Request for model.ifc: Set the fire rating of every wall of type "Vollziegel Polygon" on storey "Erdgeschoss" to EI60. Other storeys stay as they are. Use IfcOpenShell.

First a look at what the model holds.

```python
import ifcopenshell
import ifcopenshell.util.element

model = ifcopenshell.open("model.ifc")
print(model.schema)
storey = next(s for s in model.by_type("IfcBuildingStorey") if s.Name == "Erdgeschoss")
walls = [e for e in ifcopenshell.util.element.get_decomposition(storey) if e.is_a("IfcWall")]
seen = {}
for e in walls:
    element_type = ifcopenshell.util.element.get_type(e)
    key = (element_type.Name if element_type != e and element_type else None, ifcopenshell.util.element.get_pset(e, "Pset_WallCommon", "FireRating"))
    seen[key] = seen.get(key, 0) + 1
for (name, value), count in sorted(seen.items(), key=str):
    print(count, "x", name, "|", value)
```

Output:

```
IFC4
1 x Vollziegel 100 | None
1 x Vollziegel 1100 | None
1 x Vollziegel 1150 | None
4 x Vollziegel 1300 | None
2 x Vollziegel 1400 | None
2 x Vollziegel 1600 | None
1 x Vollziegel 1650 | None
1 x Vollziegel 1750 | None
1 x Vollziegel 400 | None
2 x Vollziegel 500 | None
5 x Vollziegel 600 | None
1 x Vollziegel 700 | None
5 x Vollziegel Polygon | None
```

```python
import ifcopenshell
import ifcopenshell.api.pset
import ifcopenshell.util.element

model = ifcopenshell.open("model.ifc")

storey = next(s for s in model.by_type("IfcBuildingStorey") if s.Name == "Erdgeschoss")
walls = [e for e in ifcopenshell.util.element.get_decomposition(storey) if e.is_a("IfcWall")]

count = 0
for e in walls:
    element_type = ifcopenshell.util.element.get_type(e)
    if element_type in (None, e) or element_type.Name != "Vollziegel Polygon":
        continue
    # add_pset returns the element's existing set when there is one.
    pset = ifcopenshell.api.pset.add_pset(model, product=e, name="Pset_WallCommon")
    ifcopenshell.api.pset.edit_pset(model, pset=pset, properties={"FireRating": "EI60"})
    count += 1

print(count, "walls updated")

model.write("model-out.ifc")
```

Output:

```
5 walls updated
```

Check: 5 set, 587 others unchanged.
